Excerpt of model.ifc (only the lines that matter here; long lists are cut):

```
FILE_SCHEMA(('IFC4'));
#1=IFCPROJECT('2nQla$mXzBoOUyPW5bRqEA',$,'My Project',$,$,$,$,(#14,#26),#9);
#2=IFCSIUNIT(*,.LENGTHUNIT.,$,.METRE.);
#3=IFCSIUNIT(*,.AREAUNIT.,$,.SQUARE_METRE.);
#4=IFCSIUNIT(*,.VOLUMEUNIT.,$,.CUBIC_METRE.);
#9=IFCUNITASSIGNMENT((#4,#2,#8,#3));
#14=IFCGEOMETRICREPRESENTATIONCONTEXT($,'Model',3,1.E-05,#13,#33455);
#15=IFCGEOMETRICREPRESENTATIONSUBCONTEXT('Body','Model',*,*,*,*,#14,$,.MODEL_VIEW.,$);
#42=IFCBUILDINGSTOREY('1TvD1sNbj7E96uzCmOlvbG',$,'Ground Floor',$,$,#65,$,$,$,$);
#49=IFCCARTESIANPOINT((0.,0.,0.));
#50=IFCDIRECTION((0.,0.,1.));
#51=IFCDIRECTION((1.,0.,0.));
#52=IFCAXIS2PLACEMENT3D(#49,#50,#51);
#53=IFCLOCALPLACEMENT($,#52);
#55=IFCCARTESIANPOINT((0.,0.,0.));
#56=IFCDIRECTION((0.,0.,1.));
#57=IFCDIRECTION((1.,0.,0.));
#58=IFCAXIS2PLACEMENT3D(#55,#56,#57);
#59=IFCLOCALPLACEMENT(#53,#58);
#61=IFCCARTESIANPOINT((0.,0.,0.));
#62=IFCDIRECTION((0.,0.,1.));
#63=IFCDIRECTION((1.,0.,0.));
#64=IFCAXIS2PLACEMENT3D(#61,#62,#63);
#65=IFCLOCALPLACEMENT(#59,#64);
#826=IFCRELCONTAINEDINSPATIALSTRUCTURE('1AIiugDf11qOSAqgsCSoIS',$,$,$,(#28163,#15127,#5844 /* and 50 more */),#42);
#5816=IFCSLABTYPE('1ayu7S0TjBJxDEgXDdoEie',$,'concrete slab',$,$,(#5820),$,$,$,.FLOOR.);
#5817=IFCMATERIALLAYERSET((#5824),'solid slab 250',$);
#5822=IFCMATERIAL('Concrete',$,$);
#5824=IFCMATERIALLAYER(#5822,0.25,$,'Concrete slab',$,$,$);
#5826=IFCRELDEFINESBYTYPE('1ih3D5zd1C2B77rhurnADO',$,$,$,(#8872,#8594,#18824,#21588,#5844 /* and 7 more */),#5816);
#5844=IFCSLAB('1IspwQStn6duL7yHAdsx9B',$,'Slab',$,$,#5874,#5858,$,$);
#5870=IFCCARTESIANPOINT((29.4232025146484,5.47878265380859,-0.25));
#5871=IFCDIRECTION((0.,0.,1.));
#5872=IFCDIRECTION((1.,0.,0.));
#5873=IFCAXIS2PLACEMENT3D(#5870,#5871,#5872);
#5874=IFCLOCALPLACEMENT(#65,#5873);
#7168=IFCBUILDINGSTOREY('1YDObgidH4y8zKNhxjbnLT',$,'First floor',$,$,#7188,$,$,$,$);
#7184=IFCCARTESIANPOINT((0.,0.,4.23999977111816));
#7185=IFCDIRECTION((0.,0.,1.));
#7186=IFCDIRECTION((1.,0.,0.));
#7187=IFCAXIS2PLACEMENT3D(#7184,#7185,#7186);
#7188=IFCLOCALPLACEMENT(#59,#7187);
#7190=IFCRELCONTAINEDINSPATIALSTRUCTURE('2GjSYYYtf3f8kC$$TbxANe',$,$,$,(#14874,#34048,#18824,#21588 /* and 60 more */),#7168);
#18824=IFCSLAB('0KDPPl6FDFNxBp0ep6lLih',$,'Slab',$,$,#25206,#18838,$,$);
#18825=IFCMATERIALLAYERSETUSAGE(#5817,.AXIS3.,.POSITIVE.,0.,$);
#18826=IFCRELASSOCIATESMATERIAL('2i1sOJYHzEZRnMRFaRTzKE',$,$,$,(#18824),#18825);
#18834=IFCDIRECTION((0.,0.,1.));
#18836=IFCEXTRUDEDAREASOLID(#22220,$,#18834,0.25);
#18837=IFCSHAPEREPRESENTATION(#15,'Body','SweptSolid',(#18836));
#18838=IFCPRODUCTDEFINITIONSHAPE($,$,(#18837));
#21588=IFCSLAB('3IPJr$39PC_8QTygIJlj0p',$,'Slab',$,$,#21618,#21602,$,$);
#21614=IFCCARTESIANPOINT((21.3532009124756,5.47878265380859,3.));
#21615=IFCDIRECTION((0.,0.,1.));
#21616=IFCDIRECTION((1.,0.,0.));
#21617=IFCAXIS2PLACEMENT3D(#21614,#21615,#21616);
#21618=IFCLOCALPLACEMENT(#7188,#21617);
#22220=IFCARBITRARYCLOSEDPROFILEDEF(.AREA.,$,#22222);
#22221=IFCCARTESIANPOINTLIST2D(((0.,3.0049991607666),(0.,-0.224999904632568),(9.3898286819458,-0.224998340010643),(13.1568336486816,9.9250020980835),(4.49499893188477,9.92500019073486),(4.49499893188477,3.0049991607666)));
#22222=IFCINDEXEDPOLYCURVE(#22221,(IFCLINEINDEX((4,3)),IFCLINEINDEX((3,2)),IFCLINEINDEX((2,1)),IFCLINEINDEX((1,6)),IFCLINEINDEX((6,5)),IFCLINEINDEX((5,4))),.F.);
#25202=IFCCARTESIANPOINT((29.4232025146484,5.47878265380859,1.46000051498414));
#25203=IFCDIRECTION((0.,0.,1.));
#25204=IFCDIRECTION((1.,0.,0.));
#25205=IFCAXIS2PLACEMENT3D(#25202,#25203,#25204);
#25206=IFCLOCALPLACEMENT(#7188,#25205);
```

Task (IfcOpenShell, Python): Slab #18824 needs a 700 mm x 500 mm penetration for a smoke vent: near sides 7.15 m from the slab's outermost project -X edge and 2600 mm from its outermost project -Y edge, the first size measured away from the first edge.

```python
import numpy as np
import ifcopenshell
import ifcopenshell.api.feature
import ifcopenshell.api.geometry
import ifcopenshell.api.root
import ifcopenshell.geom
import ifcopenshell.util.placement
import ifcopenshell.util.representation
import ifcopenshell.util.shape
import ifcopenshell.util.unit

model = ifcopenshell.open("model.ifc")
unit_scale = ifcopenshell.util.unit.calculate_unit_scale(model)
settings = ifcopenshell.geom.settings()


def volume(element):
    """Net volume in cubic metres, openings subtracted."""
    shape = ifcopenshell.geom.create_shape(settings, element)
    return ifcopenshell.util.shape.get_volume(shape.geometry)


slab = model.by_guid("0KDPPl6FDFNxBp0ep6lLih")
before = volume(slab)

# Extent in the slab's own axes, in metres. The edges named are its -X and -Y sides.
slab_shape = ifcopenshell.geom.create_shape(settings, slab)
vertices = ifcopenshell.util.shape.get_vertices(slab_shape.geometry)
x_min, y_min, bottom = vertices.min(axis=0)
top = vertices[:, 2].max()

opening = ifcopenshell.api.root.create_entity(model, ifc_class="IfcOpeningElement", name="Smoke vent opening", predefined_type="OPENING")
context = ifcopenshell.util.representation.get_context(model, "Model", "Body", "MODEL_VIEW")
width, depth = 0.7, 0.5
outline = [(0.0, 0.0), (width, 0.0), (width, depth), (0.0, depth), (0.0, 0.0)]
# Overshoot both faces by 50 mm so the cut is clean.
shape = ifcopenshell.api.geometry.add_slab_representation(
    model, context=context, depth=top - bottom + 0.1, polyline=outline
)
ifcopenshell.api.geometry.assign_representation(model, product=opening, representation=shape)

matrix = ifcopenshell.util.placement.get_local_placement(slab.ObjectPlacement)
matrix[:, 3] = matrix @ np.append(np.array([x_min + 7.15, y_min + 2.6, bottom - 0.05]) / unit_scale, 1.0)
ifcopenshell.api.geometry.edit_object_placement(model, product=opening, matrix=matrix, is_si=False)
ifcopenshell.api.feature.add_feature(model, feature=opening, element=slab)

after = volume(slab)

print(f"slab volume {before:.3f} -> {after:.3f} m3")

model.write("model_edited.ifc")
```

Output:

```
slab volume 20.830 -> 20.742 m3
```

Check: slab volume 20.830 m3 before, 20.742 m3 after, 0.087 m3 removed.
